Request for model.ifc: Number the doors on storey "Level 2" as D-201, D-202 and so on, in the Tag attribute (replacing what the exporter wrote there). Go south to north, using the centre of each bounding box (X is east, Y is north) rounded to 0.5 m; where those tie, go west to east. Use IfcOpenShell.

First a look at what the model holds.

```python
import ifcopenshell
import ifcopenshell.util.element
import ifcopenshell.util.placement

model = ifcopenshell.open("model.ifc")
print(model.schema)
storey = next(s for s in model.by_type("IfcBuildingStorey") if s.Name == "Level 2")
doors = [e for e in ifcopenshell.util.element.get_decomposition(storey) if e.is_a("IfcDoor")]
for e in sorted(doors, key=lambda e: e.id()):
    origin = ifcopenshell.util.placement.get_local_placement(e.ObjectPlacement)[:3, 3]
    print(e.id(), e.Tag, e.Name, origin.round(2) + 0.0, sep=" | ")
```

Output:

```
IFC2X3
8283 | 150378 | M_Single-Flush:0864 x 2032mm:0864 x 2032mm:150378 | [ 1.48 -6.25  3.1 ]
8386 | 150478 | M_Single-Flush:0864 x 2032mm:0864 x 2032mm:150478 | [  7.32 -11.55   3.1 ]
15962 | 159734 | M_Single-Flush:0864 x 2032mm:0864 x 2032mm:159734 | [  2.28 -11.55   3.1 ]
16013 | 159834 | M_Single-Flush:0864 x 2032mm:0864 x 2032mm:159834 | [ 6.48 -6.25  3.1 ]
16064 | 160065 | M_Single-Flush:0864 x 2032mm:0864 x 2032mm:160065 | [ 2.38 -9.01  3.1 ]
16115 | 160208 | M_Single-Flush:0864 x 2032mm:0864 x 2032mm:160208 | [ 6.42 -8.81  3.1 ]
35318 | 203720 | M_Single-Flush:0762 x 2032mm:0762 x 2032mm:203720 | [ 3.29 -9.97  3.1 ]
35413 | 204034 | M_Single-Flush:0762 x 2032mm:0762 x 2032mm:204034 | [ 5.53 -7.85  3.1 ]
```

```python
import ifcopenshell
import ifcopenshell.geom
import ifcopenshell.util.element
import ifcopenshell.util.shape

model = ifcopenshell.open("model.ifc")
settings = ifcopenshell.geom.settings()
settings.set("use-world-coords", True)


def centre(element):
    shape = ifcopenshell.geom.create_shape(settings, element)
    return ifcopenshell.util.shape.get_bbox_centroid(shape.geometry)


storey = next(s for s in model.by_type("IfcBuildingStorey") if s.Name == "Level 2")
doors = [e for e in ifcopenshell.util.element.get_decomposition(storey) if e.is_a("IfcDoor")]

# Insertion points can sit at a corner or the storey origin, so sort by the geometry (in metres).
centres = {e: centre(e) for e in doors}
doors.sort(key=lambda e: (round(centres[e][1] / 0.5), centres[e][0]))

for i, e in enumerate(doors, start=1):
    number = f"D-2{i:02d}"
    e.Tag = number
    print(e.id(), number)

model.write("model_updated.ifc")
```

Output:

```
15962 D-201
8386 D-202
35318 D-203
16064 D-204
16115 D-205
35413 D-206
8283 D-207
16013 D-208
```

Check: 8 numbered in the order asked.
